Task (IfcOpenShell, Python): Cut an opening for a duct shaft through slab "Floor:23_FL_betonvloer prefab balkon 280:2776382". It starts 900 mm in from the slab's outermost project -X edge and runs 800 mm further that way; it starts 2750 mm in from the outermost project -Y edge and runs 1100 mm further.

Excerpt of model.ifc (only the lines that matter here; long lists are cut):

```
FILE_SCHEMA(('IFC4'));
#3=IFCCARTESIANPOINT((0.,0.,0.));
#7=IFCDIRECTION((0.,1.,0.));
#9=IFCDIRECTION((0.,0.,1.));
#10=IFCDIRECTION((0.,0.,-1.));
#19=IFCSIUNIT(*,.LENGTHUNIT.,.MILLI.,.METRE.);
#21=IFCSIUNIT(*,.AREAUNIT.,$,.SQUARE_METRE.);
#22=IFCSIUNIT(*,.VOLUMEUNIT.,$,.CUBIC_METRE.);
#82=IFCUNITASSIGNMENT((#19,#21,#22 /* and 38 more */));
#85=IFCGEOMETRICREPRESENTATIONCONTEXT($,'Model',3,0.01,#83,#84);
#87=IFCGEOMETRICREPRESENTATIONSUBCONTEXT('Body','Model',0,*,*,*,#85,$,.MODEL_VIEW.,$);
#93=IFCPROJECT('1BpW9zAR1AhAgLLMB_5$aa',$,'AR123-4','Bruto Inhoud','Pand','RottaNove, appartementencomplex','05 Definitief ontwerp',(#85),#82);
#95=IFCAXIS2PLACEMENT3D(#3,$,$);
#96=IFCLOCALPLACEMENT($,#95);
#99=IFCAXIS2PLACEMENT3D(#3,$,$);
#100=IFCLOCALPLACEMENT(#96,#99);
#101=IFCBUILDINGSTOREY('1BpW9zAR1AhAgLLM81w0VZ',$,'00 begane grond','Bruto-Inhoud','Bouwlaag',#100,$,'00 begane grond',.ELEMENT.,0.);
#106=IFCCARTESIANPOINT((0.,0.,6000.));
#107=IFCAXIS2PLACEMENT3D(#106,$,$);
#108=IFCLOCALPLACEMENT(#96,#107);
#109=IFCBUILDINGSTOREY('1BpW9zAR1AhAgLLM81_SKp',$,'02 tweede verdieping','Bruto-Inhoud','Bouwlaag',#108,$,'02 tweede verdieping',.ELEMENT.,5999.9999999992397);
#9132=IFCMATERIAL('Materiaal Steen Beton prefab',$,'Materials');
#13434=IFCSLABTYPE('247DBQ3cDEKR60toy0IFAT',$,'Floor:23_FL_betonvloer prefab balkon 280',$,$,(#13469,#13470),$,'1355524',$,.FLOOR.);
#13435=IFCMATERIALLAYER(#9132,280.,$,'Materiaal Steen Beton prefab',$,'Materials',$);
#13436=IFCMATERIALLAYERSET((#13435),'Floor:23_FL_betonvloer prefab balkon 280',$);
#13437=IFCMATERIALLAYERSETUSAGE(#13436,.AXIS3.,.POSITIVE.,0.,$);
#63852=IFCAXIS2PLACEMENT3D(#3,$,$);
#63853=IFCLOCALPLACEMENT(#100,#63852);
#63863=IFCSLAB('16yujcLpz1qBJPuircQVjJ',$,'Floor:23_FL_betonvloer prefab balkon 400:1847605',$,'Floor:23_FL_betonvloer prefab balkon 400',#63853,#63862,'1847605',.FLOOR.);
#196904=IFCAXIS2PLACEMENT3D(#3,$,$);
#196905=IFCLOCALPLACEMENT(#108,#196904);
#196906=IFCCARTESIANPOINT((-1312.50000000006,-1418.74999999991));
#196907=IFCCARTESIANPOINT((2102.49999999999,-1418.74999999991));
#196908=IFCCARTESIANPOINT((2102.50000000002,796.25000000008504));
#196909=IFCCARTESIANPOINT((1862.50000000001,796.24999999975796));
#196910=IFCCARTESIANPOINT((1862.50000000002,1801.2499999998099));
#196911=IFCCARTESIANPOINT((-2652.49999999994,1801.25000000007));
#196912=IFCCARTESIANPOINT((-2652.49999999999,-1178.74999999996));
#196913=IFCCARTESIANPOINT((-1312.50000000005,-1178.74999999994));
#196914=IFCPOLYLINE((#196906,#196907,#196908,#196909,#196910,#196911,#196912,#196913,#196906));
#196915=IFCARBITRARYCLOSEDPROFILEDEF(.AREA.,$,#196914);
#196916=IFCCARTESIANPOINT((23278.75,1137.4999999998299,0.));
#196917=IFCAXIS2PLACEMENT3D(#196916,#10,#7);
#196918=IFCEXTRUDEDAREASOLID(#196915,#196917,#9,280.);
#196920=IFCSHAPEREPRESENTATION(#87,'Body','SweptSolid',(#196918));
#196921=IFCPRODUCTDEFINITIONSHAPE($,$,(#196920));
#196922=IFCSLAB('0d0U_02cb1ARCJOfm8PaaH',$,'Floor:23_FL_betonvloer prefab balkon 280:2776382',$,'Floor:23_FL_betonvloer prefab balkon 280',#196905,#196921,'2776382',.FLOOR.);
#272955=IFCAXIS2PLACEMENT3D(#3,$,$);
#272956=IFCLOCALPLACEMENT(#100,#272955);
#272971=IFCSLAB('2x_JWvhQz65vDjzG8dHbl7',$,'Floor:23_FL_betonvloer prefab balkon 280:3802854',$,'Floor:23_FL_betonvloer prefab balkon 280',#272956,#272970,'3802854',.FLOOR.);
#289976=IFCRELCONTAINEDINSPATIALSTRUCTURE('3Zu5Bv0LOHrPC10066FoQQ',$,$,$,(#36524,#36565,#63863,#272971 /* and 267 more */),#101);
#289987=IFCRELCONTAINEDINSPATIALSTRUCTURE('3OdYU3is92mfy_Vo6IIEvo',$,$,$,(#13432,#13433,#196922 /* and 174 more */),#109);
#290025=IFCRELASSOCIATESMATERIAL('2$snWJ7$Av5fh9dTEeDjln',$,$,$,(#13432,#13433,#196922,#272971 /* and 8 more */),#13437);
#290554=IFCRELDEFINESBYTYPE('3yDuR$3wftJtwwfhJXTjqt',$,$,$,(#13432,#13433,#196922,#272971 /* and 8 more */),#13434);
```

```python
import numpy as np
import ifcopenshell
import ifcopenshell.api.feature
import ifcopenshell.api.geometry
import ifcopenshell.api.root
import ifcopenshell.geom
import ifcopenshell.util.placement
import ifcopenshell.util.representation
import ifcopenshell.util.shape
import ifcopenshell.util.unit

model = ifcopenshell.open("model.ifc")
unit_scale = ifcopenshell.util.unit.calculate_unit_scale(model)
settings = ifcopenshell.geom.settings()


def volume(element):
    """Net volume in cubic metres, openings subtracted."""
    shape = ifcopenshell.geom.create_shape(settings, element)
    return ifcopenshell.util.shape.get_volume(shape.geometry)


slab = model.by_guid("0d0U_02cb1ARCJOfm8PaaH")
before = volume(slab)

# Extent in the slab's own axes, in metres. The edges named are its -X and -Y sides.
slab_shape = ifcopenshell.geom.create_shape(settings, slab)
vertices = ifcopenshell.util.shape.get_vertices(slab_shape.geometry)
x_min, y_min, bottom = vertices.min(axis=0)
top = vertices[:, 2].max()

opening = ifcopenshell.api.root.create_entity(model, ifc_class="IfcOpeningElement", name="Duct shaft opening", predefined_type="OPENING")
context = ifcopenshell.util.representation.get_context(model, "Model", "Body", "MODEL_VIEW")
width, depth = 0.8, 1.1
outline = [(0.0, 0.0), (width, 0.0), (width, depth), (0.0, depth), (0.0, 0.0)]
# Overshoot both faces by 50 mm so the cut is clean.
shape = ifcopenshell.api.geometry.add_slab_representation(
    model, context=context, depth=top - bottom + 0.1, polyline=outline
)
ifcopenshell.api.geometry.assign_representation(model, product=opening, representation=shape)

matrix = ifcopenshell.util.placement.get_local_placement(slab.ObjectPlacement)
matrix[:, 3] = matrix @ np.append(np.array([x_min + 0.9, y_min + 2.75, bottom - 0.05]) / unit_scale, 1.0)
ifcopenshell.api.geometry.edit_object_placement(model, product=opening, matrix=matrix, is_si=False)
ifcopenshell.api.feature.add_feature(model, feature=opening, element=slab)

after = volume(slab)

print(f"slab volume {before:.3f} -> {after:.3f} m3")

model.write("model_rev.ifc")
```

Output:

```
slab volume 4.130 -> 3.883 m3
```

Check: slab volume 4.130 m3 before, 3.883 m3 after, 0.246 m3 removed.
